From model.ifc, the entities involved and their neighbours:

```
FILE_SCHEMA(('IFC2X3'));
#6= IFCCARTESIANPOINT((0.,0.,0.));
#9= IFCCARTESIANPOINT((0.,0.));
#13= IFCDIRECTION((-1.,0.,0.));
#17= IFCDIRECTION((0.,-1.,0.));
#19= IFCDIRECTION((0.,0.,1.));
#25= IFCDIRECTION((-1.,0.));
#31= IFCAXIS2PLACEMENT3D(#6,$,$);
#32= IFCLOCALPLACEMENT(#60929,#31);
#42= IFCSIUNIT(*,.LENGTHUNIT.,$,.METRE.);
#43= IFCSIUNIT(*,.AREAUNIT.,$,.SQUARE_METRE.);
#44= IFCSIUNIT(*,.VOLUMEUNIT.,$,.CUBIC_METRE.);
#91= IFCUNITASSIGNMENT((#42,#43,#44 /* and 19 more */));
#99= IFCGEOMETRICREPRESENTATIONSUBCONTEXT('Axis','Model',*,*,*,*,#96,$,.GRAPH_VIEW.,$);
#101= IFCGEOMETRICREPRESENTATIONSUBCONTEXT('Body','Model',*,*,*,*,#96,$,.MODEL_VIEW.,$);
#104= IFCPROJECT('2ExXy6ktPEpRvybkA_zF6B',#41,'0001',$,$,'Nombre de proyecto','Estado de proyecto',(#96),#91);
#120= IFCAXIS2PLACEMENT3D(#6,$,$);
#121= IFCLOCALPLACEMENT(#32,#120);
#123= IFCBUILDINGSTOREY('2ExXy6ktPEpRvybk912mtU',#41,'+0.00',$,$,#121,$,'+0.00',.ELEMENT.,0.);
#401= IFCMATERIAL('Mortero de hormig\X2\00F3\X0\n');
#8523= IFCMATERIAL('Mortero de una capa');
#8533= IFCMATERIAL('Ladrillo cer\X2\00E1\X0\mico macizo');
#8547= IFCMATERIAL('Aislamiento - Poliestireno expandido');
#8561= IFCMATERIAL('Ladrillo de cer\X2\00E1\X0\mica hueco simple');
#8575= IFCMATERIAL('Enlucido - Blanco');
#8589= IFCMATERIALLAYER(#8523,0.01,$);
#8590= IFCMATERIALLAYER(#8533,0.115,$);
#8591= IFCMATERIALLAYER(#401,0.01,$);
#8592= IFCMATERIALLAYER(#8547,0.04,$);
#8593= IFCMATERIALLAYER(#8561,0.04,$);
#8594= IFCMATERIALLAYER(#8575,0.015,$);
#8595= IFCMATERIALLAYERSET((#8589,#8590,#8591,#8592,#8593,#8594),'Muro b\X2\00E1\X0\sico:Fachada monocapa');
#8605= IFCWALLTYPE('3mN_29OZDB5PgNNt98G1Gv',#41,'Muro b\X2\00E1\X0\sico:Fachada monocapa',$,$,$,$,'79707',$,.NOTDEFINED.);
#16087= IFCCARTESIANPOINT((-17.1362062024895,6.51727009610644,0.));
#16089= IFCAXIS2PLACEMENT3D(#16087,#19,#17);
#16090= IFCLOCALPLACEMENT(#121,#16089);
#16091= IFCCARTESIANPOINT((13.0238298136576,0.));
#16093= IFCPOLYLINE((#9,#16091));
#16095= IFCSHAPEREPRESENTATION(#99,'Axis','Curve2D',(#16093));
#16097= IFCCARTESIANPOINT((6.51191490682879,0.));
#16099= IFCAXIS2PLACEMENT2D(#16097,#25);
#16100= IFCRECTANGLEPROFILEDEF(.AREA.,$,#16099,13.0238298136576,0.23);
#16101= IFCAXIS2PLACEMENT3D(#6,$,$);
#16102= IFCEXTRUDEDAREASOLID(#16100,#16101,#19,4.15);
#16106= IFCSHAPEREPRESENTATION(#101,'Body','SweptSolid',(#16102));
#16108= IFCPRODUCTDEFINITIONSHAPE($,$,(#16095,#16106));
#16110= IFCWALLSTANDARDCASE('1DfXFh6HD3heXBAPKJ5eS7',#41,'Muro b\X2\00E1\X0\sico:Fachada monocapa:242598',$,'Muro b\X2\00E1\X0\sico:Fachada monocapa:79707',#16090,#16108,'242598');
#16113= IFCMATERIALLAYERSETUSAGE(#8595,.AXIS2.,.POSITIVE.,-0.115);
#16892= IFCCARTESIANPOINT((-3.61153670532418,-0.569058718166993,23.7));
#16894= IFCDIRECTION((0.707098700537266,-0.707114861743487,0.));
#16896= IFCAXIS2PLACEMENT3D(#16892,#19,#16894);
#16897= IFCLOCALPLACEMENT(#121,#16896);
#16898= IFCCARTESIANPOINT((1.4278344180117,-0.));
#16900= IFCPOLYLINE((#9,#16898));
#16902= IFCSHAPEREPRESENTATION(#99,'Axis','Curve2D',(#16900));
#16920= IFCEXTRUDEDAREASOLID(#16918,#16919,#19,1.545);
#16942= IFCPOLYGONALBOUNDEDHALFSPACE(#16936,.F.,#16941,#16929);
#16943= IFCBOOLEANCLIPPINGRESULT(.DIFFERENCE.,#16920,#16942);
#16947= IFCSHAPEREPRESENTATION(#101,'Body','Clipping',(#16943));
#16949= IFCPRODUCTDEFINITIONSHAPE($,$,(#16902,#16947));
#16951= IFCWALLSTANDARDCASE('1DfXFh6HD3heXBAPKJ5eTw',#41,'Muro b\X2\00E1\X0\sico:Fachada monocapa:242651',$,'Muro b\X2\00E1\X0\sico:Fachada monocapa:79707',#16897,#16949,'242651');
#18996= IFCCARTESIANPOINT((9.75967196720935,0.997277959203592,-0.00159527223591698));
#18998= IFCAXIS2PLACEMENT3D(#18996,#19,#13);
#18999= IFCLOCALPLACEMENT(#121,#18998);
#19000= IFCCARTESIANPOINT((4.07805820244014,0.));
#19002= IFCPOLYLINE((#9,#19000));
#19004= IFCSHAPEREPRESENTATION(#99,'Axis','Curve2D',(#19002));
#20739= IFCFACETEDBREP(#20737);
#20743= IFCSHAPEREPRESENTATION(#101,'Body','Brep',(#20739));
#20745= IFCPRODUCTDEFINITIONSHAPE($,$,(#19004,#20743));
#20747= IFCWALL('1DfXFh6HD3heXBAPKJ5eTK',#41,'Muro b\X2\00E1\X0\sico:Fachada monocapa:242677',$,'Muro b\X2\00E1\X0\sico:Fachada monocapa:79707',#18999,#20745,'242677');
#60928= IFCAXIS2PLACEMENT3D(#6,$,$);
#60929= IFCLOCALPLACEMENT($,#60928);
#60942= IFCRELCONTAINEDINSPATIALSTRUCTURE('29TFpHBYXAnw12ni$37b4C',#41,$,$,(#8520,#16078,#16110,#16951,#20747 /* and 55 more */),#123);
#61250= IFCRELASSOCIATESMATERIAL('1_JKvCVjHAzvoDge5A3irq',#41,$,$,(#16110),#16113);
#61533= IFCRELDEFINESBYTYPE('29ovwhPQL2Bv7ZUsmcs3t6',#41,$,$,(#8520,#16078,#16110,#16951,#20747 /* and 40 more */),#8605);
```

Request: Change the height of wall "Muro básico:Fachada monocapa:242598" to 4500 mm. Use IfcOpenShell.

```python
import ifcopenshell
import ifcopenshell.geom
import ifcopenshell.util.representation
import ifcopenshell.util.shape
import ifcopenshell.util.unit

model = ifcopenshell.open("model.ifc")
unit_scale = ifcopenshell.util.unit.calculate_unit_scale(model)
settings = ifcopenshell.geom.settings()


def volume(element):
    """Net volume in cubic metres, openings subtracted."""
    shape = ifcopenshell.geom.create_shape(settings, element)
    return ifcopenshell.util.shape.get_volume(shape.geometry)


wall = model.by_id(16110)
before = volume(wall)

body = ifcopenshell.util.representation.get_representation(wall, "Model", "Body")
solid = body.Items[0]
old_height = solid.Depth
solid.Depth = 4.5 / unit_scale
after = volume(wall)

print(f"height {old_height:g} -> {solid.Depth:g}, volume {before:.3f} -> {after:.3f} m3")

model.write("model_v2.ifc")
```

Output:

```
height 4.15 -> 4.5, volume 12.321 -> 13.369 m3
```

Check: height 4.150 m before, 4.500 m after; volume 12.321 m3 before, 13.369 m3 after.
